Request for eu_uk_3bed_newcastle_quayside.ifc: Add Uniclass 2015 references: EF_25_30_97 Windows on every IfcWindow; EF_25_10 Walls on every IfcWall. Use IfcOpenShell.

First a look at what the model holds.

```python
import ifcopenshell

model = ifcopenshell.open("eu_uk_3bed_newcastle_quayside.ifc")
print(model.schema)
print("classifications:", [c.Name for c in model.by_type("IfcClassification")])
for ifc_class in ("IfcDoor", "IfcRoof", "IfcStair", "IfcWall", "IfcWindow"):
    print(ifc_class, len(model.by_type(ifc_class)))
```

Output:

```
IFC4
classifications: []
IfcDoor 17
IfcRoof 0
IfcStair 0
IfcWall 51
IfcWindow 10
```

```python
import ifcopenshell
import ifcopenshell.api.classification

model = ifcopenshell.open("eu_uk_3bed_newcastle_quayside.ifc")

system = ifcopenshell.api.classification.add_classification(model, classification="Uniclass 2015")

codes = {
    "IfcWindow": ("EF_25_30_97", "Windows"),
    "IfcWall": ("EF_25_10", "Walls"),
}
for ifc_class, (code, name) in codes.items():
    products = model.by_type(ifc_class)
    ifcopenshell.api.classification.add_reference(
        model, products=products, classification=system, identification=code, name=name
    )
    print(code, len(products))

model.write("eu_uk_3bed_newcastle_quayside_v2.ifc")
```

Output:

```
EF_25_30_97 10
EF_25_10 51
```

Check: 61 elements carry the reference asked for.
